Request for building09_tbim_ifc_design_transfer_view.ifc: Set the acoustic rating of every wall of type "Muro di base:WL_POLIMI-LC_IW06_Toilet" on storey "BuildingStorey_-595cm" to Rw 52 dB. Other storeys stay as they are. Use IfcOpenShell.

First a look at what the model holds.

```python
import ifcopenshell
import ifcopenshell.util.element

model = ifcopenshell.open("building09_tbim_ifc_design_transfer_view.ifc")
print(model.schema)
storey = next(s for s in model.by_type("IfcBuildingStorey") if s.Name == "BuildingStorey_-595cm")
walls = [e for e in ifcopenshell.util.element.get_decomposition(storey) if e.is_a("IfcWall")]
seen = {}
for e in walls:
    element_type = ifcopenshell.util.element.get_type(e)
    key = (element_type.Name if element_type != e and element_type else None, ifcopenshell.util.element.get_pset(e, "Pset_WallCommon", "AcousticRating"))
    seen[key] = seen.get(key, 0) + 1
for (name, value), count in sorted(seen.items(), key=str):
    print(count, "x", name, "|", value)
```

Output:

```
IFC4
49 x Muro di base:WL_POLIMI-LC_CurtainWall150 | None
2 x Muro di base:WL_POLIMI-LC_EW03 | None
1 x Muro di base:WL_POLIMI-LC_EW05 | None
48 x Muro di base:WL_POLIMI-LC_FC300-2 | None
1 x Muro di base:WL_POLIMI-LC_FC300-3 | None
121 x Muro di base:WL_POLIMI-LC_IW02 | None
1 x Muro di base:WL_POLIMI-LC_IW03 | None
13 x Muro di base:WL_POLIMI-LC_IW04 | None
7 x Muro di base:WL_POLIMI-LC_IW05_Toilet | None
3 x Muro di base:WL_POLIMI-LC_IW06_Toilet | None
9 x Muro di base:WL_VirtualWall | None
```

```python
import ifcopenshell
import ifcopenshell.api.pset
import ifcopenshell.util.element

model = ifcopenshell.open("building09_tbim_ifc_design_transfer_view.ifc")

storey = next(s for s in model.by_type("IfcBuildingStorey") if s.Name == "BuildingStorey_-595cm")
walls = [e for e in ifcopenshell.util.element.get_decomposition(storey) if e.is_a("IfcWall")]

count = 0
for e in walls:
    element_type = ifcopenshell.util.element.get_type(e)
    if element_type in (None, e) or element_type.Name != "Muro di base:WL_POLIMI-LC_IW06_Toilet":
        continue
    # add_pset returns the element's existing set when there is one.
    pset = ifcopenshell.api.pset.add_pset(model, product=e, name="Pset_WallCommon")
    ifcopenshell.api.pset.edit_pset(model, pset=pset, properties={"AcousticRating": "Rw 52 dB"})
    count += 1

print(count, "walls updated")

model.write("building09_tbim_ifc_design_transfer_view_v2.ifc")
```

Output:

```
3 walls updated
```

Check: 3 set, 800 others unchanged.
